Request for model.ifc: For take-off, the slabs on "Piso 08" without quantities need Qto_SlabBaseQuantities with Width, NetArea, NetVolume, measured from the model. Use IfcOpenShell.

First a look at what the model holds.

```python
import ifcopenshell
import ifcopenshell.util.element
import ifcopenshell.util.unit

model = ifcopenshell.open("model.ifc")
print(model.schema)
for unit_type in ("LENGTHUNIT", "AREAUNIT", "VOLUMEUNIT"):
    print(unit_type, ifcopenshell.util.unit.calculate_unit_scale(model, unit_type))
storey = next(s for s in model.by_type("IfcBuildingStorey") if s.Name == "Piso 08")
slabs = [e for e in ifcopenshell.util.element.get_decomposition(storey) if e.is_a("IfcSlab")]
for e in sorted(slabs, key=lambda e: e.id()):
    print(e.id(), e.is_a(), e.Name, list(ifcopenshell.util.element.get_psets(e, qtos_only=True)), sep=" | ")
```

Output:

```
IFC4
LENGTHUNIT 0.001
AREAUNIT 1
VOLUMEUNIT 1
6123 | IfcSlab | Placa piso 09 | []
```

```python
import ifcopenshell
import ifcopenshell.api.pset
import ifcopenshell.geom
import ifcopenshell.util.element
import ifcopenshell.util.shape
import ifcopenshell.util.unit

model = ifcopenshell.open("model.ifc")
unit_scale = ifcopenshell.util.unit.calculate_unit_scale(model)
area_scale = ifcopenshell.util.unit.calculate_unit_scale(model, "AREAUNIT")
volume_scale = ifcopenshell.util.unit.calculate_unit_scale(model, "VOLUMEUNIT")
settings = ifcopenshell.geom.settings()

storey = next(s for s in model.by_type("IfcBuildingStorey") if s.Name == "Piso 08")
slabs = [e for e in ifcopenshell.util.element.get_decomposition(storey) if e.is_a("IfcSlab")]

for e in sorted(slabs, key=lambda e: e.id()):
    if ifcopenshell.util.element.get_psets(e, qtos_only=True, should_inherit=False):
        continue
    # Geometry comes back in metres, in the element's own axes.
    shape = ifcopenshell.geom.create_shape(settings, e)
    values = {
        "Width": ifcopenshell.util.shape.get_z(shape.geometry) / unit_scale,
        "NetArea": ifcopenshell.util.shape.get_footprint_area(shape.geometry) / area_scale,
        "NetVolume": ifcopenshell.util.shape.get_volume(shape.geometry) / volume_scale,
    }
    qto = ifcopenshell.api.pset.add_qto(model, product=e, name="Qto_SlabBaseQuantities")
    ifcopenshell.api.pset.edit_qto(model, qto=qto, properties=values)
    print(e.id(), {k: round(v, 3) for k, v in values.items()})

model.write("model_rev.ifc")
```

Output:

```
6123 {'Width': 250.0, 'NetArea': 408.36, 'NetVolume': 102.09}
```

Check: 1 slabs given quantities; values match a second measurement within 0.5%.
